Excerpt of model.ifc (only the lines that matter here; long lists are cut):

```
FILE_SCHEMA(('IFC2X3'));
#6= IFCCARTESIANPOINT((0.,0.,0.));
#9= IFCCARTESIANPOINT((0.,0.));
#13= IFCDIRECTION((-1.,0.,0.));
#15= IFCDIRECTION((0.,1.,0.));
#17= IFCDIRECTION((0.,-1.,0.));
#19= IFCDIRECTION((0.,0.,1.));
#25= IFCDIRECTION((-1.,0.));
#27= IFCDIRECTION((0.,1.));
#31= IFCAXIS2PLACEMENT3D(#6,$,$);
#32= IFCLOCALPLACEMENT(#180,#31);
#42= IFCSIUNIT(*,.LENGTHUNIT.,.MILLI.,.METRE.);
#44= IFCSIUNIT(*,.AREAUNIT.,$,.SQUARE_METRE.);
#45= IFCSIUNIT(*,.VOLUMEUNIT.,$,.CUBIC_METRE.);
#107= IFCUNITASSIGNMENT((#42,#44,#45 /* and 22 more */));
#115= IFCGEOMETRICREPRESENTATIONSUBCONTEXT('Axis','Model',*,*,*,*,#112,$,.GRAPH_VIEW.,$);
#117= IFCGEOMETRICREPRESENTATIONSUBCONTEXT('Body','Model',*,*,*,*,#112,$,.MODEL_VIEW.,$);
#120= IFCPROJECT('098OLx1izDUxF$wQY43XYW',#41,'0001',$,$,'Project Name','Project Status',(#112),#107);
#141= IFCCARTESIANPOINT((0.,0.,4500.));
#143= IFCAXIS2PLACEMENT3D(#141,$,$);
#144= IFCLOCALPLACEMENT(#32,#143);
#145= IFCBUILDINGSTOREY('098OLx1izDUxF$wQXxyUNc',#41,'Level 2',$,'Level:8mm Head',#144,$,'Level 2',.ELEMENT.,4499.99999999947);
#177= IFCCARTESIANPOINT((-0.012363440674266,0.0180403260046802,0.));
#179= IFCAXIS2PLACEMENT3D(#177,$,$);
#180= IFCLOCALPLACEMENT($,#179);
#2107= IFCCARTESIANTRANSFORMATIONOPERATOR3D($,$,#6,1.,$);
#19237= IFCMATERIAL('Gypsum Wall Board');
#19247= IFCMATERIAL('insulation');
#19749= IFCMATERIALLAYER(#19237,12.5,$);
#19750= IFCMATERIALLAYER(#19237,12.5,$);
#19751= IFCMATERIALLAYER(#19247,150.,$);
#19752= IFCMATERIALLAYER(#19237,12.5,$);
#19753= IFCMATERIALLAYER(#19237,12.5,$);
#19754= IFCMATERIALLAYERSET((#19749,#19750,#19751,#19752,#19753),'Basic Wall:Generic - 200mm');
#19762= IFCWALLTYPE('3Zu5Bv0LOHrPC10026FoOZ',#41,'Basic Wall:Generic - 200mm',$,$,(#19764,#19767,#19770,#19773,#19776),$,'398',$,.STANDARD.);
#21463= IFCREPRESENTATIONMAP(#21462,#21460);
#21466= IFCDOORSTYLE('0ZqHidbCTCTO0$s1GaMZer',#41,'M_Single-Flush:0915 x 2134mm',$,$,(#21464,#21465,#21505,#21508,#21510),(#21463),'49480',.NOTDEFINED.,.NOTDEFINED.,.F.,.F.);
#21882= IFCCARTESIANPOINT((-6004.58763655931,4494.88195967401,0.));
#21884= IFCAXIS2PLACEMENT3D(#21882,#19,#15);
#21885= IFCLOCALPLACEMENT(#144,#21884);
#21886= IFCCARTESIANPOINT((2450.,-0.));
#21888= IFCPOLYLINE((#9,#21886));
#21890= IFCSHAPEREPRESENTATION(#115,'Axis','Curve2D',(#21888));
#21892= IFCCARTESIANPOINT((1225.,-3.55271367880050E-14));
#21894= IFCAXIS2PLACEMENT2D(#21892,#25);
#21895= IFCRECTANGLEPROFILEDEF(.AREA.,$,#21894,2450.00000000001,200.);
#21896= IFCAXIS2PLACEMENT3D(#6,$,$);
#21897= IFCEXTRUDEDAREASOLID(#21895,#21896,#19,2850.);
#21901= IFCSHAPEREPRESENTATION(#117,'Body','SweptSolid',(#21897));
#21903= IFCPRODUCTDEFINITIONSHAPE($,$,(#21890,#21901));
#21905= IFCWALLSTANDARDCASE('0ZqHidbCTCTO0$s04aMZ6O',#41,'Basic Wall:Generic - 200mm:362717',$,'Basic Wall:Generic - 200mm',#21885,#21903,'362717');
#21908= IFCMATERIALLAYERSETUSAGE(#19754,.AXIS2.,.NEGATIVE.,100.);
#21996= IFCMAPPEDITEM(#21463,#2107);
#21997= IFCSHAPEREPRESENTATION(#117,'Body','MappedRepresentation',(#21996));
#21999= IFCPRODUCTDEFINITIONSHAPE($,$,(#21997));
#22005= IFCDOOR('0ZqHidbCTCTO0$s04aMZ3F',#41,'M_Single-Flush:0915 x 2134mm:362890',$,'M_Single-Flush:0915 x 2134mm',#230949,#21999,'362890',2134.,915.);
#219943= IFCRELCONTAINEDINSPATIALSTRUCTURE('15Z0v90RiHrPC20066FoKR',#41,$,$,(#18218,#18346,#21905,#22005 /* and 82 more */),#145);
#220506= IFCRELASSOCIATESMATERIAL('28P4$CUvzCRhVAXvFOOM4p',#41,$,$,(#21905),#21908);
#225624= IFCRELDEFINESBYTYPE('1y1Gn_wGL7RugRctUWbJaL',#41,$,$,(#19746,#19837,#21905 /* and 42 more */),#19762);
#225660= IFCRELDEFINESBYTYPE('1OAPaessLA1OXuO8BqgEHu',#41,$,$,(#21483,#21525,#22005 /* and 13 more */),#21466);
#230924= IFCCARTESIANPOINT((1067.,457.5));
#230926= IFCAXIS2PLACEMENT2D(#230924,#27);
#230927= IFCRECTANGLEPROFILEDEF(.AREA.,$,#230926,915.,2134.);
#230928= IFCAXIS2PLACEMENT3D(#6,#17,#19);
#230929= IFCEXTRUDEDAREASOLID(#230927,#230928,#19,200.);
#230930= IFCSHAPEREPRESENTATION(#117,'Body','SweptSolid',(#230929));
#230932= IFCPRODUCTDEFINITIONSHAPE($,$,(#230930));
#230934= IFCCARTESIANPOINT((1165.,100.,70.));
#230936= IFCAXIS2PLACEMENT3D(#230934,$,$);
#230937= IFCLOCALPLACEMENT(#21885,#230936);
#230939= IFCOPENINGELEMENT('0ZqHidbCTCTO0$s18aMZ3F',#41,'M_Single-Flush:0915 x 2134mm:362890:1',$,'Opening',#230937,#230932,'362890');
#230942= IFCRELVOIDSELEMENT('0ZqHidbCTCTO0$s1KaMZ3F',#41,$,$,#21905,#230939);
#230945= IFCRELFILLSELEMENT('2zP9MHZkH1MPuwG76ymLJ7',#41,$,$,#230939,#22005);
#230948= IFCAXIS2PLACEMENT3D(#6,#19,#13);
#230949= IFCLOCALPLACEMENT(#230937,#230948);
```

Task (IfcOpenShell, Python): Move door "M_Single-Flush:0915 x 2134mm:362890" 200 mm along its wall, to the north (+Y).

```python
import ifcopenshell
import ifcopenshell.api.geometry
import ifcopenshell.util.placement
import ifcopenshell.util.unit

model = ifcopenshell.open("model.ifc")
unit_scale = ifcopenshell.util.unit.calculate_unit_scale(model)

door = model.by_id(22005)
opening = door.FillsVoids[0].RelatingOpeningElement
wall = opening.VoidsElements[0].RelatingBuildingElement

wall_matrix = ifcopenshell.util.placement.get_local_placement(wall.ObjectPlacement)
shift = wall_matrix[:3, 0] * 0.2 / unit_scale
before = ifcopenshell.util.placement.get_local_placement(door.ObjectPlacement)[:3, 3].copy()

# The door is placed relative to its opening, so it follows when the opening moves.
matrix = ifcopenshell.util.placement.get_local_placement(opening.ObjectPlacement)
matrix[:3, 3] += shift
ifcopenshell.api.geometry.edit_object_placement(
    model, product=opening, matrix=matrix, is_si=False, should_transform_children=True
)

after = ifcopenshell.util.placement.get_local_placement(door.ObjectPlacement)[:3, 3]
print("door moved by", (after - before).round(3) + 0.0)

model.write("model_edited.ifc")
```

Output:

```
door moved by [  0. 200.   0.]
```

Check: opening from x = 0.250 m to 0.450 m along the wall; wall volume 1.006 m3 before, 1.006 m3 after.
